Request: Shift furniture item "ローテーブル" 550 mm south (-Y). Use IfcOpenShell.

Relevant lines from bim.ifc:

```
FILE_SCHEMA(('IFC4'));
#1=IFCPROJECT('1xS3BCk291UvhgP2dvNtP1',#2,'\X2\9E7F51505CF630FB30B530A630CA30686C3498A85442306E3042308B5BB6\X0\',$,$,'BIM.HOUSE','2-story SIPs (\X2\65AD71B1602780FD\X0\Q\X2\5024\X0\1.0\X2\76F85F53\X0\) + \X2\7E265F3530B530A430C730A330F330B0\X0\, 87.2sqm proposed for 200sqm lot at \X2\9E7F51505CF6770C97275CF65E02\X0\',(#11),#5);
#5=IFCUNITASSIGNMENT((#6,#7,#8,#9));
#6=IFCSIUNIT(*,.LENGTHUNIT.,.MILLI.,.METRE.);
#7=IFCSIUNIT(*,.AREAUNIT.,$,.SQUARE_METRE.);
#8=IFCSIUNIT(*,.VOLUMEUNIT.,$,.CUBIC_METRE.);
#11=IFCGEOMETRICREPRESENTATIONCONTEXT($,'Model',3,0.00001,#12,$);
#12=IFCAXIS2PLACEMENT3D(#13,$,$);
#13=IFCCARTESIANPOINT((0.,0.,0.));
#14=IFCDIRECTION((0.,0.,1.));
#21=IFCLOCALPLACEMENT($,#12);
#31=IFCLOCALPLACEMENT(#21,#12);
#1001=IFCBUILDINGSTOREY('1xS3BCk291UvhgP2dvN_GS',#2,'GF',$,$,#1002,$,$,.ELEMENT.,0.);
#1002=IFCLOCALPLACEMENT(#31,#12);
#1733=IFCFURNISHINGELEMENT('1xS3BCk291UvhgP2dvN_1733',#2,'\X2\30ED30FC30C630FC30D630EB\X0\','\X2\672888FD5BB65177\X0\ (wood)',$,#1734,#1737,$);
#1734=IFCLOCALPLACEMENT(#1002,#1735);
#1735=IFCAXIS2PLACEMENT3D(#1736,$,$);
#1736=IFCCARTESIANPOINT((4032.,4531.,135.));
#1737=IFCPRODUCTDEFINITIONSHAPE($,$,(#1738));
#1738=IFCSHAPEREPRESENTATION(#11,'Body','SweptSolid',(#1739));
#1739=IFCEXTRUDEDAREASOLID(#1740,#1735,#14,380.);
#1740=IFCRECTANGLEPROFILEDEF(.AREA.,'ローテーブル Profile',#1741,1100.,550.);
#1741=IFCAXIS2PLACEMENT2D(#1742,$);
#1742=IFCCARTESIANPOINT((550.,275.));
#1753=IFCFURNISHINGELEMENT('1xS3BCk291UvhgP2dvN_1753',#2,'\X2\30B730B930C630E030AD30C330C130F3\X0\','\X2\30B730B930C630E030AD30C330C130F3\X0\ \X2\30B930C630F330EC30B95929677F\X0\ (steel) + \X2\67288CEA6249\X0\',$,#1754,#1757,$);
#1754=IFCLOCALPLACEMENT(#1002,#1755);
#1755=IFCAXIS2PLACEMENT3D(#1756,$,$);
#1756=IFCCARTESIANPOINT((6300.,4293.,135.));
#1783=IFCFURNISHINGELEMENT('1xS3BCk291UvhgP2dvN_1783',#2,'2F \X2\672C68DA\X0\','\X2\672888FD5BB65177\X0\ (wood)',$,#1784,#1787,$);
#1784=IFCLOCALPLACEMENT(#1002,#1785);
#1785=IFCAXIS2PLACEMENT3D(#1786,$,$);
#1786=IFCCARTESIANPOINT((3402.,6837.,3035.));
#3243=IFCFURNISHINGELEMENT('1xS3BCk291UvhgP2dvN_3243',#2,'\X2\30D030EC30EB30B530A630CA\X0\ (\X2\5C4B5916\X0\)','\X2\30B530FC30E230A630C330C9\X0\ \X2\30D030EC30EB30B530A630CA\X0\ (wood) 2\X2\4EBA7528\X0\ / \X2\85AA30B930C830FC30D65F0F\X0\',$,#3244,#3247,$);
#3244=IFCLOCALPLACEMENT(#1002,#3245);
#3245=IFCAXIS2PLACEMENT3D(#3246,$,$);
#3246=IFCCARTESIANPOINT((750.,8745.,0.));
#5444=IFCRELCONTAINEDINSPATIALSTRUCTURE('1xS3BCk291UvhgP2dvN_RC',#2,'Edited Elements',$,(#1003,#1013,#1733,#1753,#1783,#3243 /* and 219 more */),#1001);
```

```python
import ifcopenshell
import ifcopenshell.api.geometry
import ifcopenshell.util.placement

model = ifcopenshell.open("bim.ifc")

item = model.by_guid("1xS3BCk291UvhgP2dvN_1733")
matrix = ifcopenshell.util.placement.get_local_placement(item.ObjectPlacement)
matrix[1, 3] -= 550.0
ifcopenshell.api.geometry.edit_object_placement(model, product=item, matrix=matrix, is_si=False)

print(ifcopenshell.util.placement.get_local_placement(item.ObjectPlacement).round(3) + 0.0)

model.write("bim-out.ifc")
```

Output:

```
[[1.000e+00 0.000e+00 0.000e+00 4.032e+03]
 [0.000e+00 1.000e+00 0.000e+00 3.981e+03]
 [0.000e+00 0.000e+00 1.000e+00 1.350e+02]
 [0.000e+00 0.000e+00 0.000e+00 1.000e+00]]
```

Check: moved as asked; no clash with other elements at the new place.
